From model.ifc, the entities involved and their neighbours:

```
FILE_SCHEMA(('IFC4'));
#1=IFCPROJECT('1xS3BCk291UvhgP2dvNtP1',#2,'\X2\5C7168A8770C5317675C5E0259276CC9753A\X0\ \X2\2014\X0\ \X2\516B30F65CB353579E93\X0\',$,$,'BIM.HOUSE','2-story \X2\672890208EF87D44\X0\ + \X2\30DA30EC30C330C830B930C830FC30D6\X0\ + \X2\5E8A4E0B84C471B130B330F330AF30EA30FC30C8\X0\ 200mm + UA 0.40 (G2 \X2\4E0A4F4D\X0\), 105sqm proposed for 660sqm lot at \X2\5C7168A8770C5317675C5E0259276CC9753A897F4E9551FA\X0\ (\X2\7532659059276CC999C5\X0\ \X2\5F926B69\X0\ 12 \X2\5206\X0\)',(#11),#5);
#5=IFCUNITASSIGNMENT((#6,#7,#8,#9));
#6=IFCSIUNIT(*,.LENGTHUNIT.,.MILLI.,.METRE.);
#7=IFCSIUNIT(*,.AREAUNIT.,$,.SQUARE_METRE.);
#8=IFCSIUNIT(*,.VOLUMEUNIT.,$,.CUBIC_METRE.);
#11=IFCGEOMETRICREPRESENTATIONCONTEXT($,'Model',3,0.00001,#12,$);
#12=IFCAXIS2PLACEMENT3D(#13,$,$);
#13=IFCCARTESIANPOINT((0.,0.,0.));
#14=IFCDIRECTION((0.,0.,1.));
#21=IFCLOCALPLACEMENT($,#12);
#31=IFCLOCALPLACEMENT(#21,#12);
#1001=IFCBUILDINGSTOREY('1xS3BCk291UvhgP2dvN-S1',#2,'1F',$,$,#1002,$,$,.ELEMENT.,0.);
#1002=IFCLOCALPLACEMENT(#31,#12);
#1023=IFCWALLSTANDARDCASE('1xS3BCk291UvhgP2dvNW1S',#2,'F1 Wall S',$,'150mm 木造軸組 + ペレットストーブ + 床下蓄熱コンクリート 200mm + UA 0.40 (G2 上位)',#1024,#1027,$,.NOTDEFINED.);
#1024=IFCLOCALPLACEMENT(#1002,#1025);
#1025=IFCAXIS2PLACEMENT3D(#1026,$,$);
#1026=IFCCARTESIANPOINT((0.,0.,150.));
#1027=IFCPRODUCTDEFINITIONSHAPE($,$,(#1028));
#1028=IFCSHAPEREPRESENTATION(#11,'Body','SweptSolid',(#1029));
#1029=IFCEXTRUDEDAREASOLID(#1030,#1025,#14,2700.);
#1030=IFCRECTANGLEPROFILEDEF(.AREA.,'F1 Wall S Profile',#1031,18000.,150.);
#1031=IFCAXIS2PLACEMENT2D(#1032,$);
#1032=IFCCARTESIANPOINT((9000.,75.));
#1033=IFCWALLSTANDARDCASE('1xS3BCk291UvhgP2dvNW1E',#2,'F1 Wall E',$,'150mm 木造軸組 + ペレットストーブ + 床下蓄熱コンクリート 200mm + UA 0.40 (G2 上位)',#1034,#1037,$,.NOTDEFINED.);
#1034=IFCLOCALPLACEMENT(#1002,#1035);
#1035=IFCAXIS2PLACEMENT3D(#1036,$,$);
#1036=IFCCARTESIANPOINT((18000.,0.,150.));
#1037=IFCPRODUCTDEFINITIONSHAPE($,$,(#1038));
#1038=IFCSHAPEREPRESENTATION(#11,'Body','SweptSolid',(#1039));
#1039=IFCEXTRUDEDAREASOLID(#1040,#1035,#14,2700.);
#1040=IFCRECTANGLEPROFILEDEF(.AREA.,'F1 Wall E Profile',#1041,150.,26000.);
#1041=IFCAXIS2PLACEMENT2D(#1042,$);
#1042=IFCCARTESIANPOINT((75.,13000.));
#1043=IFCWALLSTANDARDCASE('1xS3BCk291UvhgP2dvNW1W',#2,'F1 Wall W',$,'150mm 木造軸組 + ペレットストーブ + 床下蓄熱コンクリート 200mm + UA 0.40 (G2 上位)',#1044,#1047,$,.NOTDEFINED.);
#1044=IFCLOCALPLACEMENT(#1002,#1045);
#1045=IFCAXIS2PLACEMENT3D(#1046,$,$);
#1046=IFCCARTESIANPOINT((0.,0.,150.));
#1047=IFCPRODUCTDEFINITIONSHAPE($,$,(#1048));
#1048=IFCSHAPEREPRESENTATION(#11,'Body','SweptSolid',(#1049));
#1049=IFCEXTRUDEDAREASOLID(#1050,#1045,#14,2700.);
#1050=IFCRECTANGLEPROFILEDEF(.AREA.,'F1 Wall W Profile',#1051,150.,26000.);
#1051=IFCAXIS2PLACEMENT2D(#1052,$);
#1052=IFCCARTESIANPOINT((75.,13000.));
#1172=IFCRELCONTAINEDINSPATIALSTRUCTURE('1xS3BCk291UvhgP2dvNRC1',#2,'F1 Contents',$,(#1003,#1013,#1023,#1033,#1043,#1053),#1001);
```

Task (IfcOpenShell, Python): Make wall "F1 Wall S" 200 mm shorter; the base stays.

```python
import ifcopenshell
import ifcopenshell.geom
import ifcopenshell.util.shape
import ifcopenshell.util.unit

model = ifcopenshell.open("model.ifc")
unit_scale = ifcopenshell.util.unit.calculate_unit_scale(model)
settings = ifcopenshell.geom.settings()


def volume(element):
    """Net volume in cubic metres, openings subtracted."""
    shape = ifcopenshell.geom.create_shape(settings, element)
    return ifcopenshell.util.shape.get_volume(shape.geometry)


wall = model.by_guid("1xS3BCk291UvhgP2dvNW1S")
before = volume(wall)

body = next(r for r in wall.Representation.Representations if r.RepresentationIdentifier == "Body")
solid = body.Items[0]
old_height = solid.Depth
solid.Depth -= 0.2 / unit_scale
after = volume(wall)

print(f"height {old_height:g} -> {solid.Depth:g}, volume {before:.3f} -> {after:.3f} m3")

model.write("model_updated.ifc")
```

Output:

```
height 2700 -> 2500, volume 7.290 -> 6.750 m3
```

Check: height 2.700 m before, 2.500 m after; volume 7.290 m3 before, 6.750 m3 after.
